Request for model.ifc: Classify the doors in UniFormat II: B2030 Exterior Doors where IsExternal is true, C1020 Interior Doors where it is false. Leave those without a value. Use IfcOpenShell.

First a look at what the model holds.

```python
import ifcopenshell
import ifcopenshell.util.element

model = ifcopenshell.open("model.ifc")
print(model.schema)
print("classifications:", [c.Name for c in model.by_type("IfcClassification")])
values = [ifcopenshell.util.element.get_pset(e, "Pset_DoorCommon", "IsExternal") for e in model.by_type("IfcDoor")]
for value in (True, False, None):
    print("IsExternal", value, values.count(value))
```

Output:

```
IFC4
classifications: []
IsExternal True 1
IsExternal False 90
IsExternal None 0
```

```python
import ifcopenshell
import ifcopenshell.api.classification
import ifcopenshell.util.element

model = ifcopenshell.open("model.ifc")

system = ifcopenshell.api.classification.add_classification(model, classification="UniFormat II")

doors = model.by_type("IfcDoor")
external = {e: ifcopenshell.util.element.get_pset(e, "Pset_DoorCommon", "IsExternal") for e in doors}
for flag, code, name in ((True, "B2030", "Exterior Doors"), (False, "C1020", "Interior Doors")):
    products = [e for e in doors if external[e] is flag]
    ifcopenshell.api.classification.add_reference(
        model, products=products, classification=system, identification=code, name=name
    )
    print(code, len(products))

model.write("model_updated.ifc")
```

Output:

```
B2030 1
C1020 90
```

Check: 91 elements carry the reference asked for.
